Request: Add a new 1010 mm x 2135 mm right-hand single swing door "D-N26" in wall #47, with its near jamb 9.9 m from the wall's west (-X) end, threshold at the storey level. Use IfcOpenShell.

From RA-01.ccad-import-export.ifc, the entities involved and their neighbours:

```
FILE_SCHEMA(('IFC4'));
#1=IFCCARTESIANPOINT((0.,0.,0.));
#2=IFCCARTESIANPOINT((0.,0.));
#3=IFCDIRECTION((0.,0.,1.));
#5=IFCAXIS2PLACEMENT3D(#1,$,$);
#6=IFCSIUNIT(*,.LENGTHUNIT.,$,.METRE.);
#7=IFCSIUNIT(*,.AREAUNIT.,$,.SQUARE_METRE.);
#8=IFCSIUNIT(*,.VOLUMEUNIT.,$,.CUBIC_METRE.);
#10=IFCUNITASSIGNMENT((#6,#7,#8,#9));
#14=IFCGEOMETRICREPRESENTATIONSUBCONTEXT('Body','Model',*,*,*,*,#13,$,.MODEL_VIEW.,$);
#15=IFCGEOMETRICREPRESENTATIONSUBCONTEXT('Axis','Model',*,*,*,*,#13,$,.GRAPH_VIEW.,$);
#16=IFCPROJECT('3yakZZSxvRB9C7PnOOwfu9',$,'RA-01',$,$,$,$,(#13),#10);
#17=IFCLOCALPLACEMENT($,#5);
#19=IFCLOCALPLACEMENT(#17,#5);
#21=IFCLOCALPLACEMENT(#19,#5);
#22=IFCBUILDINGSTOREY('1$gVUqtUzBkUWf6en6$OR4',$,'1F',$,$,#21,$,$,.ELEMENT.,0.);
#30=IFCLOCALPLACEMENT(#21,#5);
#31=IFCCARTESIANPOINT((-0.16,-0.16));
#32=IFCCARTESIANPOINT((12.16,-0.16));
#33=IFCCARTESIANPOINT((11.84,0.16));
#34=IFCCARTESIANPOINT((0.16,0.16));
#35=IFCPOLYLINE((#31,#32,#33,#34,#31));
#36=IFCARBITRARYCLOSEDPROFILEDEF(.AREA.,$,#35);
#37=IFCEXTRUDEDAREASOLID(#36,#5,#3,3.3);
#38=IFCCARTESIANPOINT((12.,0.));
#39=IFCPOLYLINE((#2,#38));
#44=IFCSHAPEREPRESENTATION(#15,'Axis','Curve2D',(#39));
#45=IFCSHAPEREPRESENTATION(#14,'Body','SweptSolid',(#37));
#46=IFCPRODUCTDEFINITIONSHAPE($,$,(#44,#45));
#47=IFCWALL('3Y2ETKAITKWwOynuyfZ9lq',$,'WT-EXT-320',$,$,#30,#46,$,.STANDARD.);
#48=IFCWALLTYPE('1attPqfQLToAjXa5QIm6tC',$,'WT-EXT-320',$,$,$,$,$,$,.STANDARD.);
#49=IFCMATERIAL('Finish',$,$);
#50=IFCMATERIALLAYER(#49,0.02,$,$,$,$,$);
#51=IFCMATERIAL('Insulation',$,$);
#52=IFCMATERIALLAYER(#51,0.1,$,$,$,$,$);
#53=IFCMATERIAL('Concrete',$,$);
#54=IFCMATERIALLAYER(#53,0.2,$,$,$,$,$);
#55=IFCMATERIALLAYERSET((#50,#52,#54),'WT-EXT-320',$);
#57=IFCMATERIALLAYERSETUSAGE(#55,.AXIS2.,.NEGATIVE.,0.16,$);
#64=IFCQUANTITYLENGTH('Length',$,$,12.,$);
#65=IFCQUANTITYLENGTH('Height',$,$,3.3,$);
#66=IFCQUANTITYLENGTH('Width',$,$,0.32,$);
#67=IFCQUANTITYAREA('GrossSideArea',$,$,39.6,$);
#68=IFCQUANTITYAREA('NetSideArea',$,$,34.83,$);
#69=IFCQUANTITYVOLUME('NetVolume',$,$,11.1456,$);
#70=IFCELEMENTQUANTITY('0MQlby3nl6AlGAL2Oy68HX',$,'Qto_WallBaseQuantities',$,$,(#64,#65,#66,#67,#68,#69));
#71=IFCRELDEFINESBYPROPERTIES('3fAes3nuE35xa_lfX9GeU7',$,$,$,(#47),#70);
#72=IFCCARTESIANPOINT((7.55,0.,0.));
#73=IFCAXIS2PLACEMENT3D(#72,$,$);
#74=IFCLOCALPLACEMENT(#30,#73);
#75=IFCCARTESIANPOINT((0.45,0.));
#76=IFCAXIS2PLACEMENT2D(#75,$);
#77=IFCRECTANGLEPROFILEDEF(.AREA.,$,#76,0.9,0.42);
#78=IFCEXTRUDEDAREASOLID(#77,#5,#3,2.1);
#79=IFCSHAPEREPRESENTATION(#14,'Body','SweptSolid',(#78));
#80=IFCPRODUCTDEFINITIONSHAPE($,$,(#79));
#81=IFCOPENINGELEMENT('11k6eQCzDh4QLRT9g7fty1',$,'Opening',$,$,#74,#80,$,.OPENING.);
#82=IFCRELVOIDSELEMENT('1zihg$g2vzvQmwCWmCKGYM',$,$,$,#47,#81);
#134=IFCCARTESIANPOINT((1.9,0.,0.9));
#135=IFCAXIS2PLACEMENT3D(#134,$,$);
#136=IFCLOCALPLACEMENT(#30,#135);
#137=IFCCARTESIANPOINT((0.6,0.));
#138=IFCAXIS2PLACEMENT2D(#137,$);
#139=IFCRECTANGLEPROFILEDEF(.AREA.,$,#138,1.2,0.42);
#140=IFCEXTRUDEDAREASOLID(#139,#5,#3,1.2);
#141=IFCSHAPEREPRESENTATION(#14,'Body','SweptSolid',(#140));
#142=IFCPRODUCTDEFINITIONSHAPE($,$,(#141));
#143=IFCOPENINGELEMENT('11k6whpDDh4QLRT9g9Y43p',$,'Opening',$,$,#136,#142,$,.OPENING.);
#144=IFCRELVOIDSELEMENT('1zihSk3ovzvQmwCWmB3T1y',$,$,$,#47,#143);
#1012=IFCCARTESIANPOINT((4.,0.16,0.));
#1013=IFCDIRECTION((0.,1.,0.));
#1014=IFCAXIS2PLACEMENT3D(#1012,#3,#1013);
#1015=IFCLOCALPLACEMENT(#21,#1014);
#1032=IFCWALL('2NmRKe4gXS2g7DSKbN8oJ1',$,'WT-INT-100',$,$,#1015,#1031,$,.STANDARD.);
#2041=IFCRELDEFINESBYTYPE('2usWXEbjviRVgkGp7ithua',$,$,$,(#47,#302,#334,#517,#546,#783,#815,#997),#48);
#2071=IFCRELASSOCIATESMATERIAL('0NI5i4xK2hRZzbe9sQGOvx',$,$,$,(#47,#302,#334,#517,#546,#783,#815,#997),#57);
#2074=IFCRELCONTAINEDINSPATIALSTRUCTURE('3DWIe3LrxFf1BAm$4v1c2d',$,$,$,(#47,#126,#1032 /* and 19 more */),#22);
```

```python
import numpy as np
import ifcopenshell
import ifcopenshell.api.feature
import ifcopenshell.api.geometry
import ifcopenshell.api.pset
import ifcopenshell.api.root
import ifcopenshell.api.spatial
import ifcopenshell.geom
import ifcopenshell.util.element
import ifcopenshell.util.placement
import ifcopenshell.util.representation
import ifcopenshell.util.shape
import ifcopenshell.util.unit

model = ifcopenshell.open("RA-01.ccad-import-export.ifc")
unit_scale = ifcopenshell.util.unit.calculate_unit_scale(model)
area_scale = ifcopenshell.util.unit.calculate_unit_scale(model, "AREAUNIT")
volume_scale = ifcopenshell.util.unit.calculate_unit_scale(model, "VOLUMEUNIT")
settings = ifcopenshell.geom.settings()


def volume(element):
    """Net volume in cubic metres, openings subtracted."""
    shape = ifcopenshell.geom.create_shape(settings, element)
    return ifcopenshell.util.shape.get_volume(shape.geometry)


wall = model.by_guid("3Y2ETKAITKWwOynuyfZ9lq")
storey = ifcopenshell.util.element.get_container(wall, ifc_class="IfcBuildingStorey")
context = ifcopenshell.util.representation.get_context(model, "Model", "Body", "MODEL_VIEW")
before = volume(wall)

width, height, from_end, sill = 1.01, 2.135, 9.9, 0.0  # metres

# The wall runs along its own X axis, and the end named is its -X end.
wall_shape = ifcopenshell.geom.create_shape(settings, wall)
x, y, z = ifcopenshell.util.shape.get_vertices(wall_shape.geometry).T
start = x.min() + from_end
face, thickness = float(y.min()), float(y.max() - y.min())
wall_matrix = ifcopenshell.util.placement.get_local_placement(wall.ObjectPlacement)
level = ifcopenshell.util.placement.get_local_placement(storey.ObjectPlacement)[2, 3]


def in_wall(x, y):
    """Placement at x, y metres in the wall's axes, at sill height."""
    matrix = wall_matrix.copy()
    matrix[:, 3] = wall_matrix @ np.array([x / unit_scale, y / unit_scale, 0.0, 1.0])
    matrix[2, 3] = level + sill / unit_scale
    return matrix


# Opening: a box that overshoots both wall faces by 50 mm.
opening = ifcopenshell.api.root.create_entity(model, ifc_class="IfcOpeningElement", predefined_type="OPENING")
box = ifcopenshell.api.geometry.add_wall_representation(
    model, context=context, length=width, height=height, thickness=thickness + 0.1
)
ifcopenshell.api.geometry.assign_representation(model, product=opening, representation=box)
ifcopenshell.api.geometry.edit_object_placement(model, product=opening, matrix=in_wall(start, face - 0.05), is_si=False)
ifcopenshell.api.feature.add_feature(model, feature=opening, element=wall)

door = ifcopenshell.api.root.create_entity(model, ifc_class="IfcDoor", name="D-N26", predefined_type="DOOR")
door.OverallWidth, door.OverallHeight = width / unit_scale, height / unit_scale
door.OperationType = "SINGLE_SWING_RIGHT"
body = ifcopenshell.api.geometry.add_door_representation(
    model,
    context=context,
    overall_width=door.OverallWidth,
    overall_height=door.OverallHeight,
    operation_type="SINGLE_SWING_RIGHT",
    lining_properties={"LiningDepth": thickness / unit_scale, "ThresholdDepth": thickness / unit_scale},
)
ifcopenshell.api.geometry.assign_representation(model, product=door, representation=body)
ifcopenshell.api.spatial.assign_container(model, products=[door], relating_structure=storey)
ifcopenshell.api.feature.add_filling(model, opening=opening, element=door)

# The lining spans the wall, so the door starts at the wall face.
ifcopenshell.api.geometry.edit_object_placement(model, product=door, matrix=in_wall(start, face), is_si=False)

after = volume(wall)

# Update the wall's stored quantities.
qto = model.by_id(ifcopenshell.util.element.get_pset(wall, "Qto_WallBaseQuantities", should_inherit=False)["id"])
ifcopenshell.api.pset.edit_qto(model, qto=qto, properties={
    "NetSideArea": after / thickness / area_scale,
    "NetVolume": after / volume_scale,
})

print(f"wall volume {before:.3f} -> {after:.3f} m3")

model.write("RA-01.ccad-import-export-out.ifc")
```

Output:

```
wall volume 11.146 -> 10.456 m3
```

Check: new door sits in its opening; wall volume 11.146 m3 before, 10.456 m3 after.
